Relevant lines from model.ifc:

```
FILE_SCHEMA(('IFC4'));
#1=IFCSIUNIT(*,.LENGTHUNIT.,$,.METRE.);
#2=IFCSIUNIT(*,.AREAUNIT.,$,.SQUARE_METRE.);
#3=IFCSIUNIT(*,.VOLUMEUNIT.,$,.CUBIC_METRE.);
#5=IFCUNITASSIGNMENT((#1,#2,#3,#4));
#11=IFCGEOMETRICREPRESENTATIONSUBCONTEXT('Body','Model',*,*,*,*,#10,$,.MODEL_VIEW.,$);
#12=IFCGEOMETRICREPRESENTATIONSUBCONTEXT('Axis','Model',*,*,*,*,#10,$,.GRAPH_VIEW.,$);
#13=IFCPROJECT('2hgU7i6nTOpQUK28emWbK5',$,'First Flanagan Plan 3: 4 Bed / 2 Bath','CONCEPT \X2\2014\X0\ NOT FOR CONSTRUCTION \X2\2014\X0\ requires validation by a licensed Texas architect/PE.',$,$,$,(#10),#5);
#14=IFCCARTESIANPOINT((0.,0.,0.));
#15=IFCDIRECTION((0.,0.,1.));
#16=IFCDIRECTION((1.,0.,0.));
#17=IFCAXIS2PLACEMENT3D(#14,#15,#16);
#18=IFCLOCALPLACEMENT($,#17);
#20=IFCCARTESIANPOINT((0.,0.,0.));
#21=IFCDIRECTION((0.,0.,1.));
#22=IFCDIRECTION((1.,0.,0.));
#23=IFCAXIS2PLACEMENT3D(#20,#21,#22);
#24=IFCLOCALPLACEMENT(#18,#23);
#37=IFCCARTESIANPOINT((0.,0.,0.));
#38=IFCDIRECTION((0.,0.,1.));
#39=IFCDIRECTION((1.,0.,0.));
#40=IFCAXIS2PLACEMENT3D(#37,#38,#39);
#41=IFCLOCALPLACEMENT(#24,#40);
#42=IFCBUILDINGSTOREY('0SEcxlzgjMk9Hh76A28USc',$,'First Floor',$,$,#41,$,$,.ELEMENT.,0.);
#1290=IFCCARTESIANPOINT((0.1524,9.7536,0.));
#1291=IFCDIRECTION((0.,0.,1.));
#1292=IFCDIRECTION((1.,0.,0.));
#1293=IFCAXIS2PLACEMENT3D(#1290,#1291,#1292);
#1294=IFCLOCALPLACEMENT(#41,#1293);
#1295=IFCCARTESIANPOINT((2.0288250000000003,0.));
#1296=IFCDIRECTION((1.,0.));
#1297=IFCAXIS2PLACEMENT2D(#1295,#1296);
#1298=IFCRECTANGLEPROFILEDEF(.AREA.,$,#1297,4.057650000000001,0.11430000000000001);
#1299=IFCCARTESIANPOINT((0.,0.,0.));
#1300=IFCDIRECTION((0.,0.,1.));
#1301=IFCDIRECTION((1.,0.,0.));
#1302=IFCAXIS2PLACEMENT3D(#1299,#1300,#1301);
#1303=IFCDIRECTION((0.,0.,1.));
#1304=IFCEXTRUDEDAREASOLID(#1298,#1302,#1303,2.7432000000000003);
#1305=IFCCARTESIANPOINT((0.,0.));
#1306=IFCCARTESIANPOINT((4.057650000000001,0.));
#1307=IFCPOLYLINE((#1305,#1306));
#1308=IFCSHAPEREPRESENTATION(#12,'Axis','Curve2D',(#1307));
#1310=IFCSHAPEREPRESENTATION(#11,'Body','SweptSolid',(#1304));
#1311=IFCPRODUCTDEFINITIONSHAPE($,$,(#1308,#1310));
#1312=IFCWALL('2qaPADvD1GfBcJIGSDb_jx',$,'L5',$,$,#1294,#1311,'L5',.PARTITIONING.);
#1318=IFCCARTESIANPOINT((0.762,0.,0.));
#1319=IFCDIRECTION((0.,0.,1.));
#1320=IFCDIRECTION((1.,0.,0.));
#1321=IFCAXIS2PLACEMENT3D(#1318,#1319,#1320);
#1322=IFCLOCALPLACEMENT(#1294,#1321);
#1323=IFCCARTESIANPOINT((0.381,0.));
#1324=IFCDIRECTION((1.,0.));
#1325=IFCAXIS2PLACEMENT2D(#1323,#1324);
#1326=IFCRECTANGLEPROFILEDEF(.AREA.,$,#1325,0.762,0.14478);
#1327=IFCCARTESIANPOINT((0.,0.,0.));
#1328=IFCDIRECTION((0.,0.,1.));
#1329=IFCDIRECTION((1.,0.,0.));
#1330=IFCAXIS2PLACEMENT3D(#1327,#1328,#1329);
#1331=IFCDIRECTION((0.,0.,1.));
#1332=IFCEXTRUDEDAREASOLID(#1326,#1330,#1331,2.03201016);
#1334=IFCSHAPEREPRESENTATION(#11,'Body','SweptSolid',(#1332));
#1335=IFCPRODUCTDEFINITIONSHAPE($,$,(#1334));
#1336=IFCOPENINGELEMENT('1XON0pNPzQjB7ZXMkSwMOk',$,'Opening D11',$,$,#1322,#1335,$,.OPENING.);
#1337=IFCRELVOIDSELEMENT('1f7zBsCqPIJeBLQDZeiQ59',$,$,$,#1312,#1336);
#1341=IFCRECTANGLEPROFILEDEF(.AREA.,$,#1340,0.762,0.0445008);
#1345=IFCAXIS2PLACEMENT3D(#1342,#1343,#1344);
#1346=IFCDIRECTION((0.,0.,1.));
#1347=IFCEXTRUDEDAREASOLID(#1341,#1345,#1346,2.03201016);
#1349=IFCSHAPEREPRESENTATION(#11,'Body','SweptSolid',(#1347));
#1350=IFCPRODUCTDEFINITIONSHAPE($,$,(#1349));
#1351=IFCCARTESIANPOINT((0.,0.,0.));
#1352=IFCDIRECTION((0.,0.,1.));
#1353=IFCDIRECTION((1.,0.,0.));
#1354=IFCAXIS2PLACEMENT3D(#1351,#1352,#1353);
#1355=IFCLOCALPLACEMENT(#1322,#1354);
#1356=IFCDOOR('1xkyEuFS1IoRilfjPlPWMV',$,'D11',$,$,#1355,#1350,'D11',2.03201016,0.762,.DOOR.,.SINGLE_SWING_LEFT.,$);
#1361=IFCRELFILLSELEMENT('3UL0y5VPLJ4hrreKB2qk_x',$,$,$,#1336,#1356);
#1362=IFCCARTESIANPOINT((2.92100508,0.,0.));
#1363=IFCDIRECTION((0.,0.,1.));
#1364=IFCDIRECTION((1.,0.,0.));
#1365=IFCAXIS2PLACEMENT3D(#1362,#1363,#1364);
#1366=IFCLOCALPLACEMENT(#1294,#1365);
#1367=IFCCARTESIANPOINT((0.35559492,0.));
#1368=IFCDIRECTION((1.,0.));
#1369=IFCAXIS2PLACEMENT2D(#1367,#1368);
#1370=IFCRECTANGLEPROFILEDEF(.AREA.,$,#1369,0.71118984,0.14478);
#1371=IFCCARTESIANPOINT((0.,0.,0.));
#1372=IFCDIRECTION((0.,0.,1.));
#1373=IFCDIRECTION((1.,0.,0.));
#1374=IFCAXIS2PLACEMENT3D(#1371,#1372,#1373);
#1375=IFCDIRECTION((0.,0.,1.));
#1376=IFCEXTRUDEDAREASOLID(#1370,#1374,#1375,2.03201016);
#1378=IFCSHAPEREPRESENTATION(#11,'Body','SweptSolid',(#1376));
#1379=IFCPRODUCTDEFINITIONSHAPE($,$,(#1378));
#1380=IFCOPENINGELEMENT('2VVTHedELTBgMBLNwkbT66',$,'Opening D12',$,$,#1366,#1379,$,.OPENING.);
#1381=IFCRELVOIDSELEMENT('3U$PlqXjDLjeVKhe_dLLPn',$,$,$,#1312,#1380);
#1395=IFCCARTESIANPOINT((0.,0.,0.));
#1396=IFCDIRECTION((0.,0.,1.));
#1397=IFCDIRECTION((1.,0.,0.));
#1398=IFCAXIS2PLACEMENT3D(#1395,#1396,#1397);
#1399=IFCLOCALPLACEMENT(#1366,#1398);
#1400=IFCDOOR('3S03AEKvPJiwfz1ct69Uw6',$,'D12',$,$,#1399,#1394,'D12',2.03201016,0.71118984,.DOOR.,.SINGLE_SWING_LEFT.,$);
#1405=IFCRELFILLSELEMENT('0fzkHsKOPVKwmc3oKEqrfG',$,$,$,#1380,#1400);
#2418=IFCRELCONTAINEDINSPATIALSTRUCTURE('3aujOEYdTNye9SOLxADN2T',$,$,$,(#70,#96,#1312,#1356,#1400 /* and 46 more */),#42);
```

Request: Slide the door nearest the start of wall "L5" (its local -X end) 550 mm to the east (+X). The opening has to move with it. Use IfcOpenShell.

```python
import ifcopenshell
import ifcopenshell.api.geometry
import ifcopenshell.util.placement
import ifcopenshell.util.unit

model = ifcopenshell.open("model.ifc")
unit_scale = ifcopenshell.util.unit.calculate_unit_scale(model)

door = model.by_id(1356)
opening = door.FillsVoids[0].RelatingOpeningElement
wall = opening.VoidsElements[0].RelatingBuildingElement

wall_matrix = ifcopenshell.util.placement.get_local_placement(wall.ObjectPlacement)
shift = wall_matrix[:3, 0] * 0.55 / unit_scale
before = ifcopenshell.util.placement.get_local_placement(door.ObjectPlacement)[:3, 3].copy()

# The door is placed relative to its opening, so it follows when the opening moves.
matrix = ifcopenshell.util.placement.get_local_placement(opening.ObjectPlacement)
matrix[:3, 3] += shift
ifcopenshell.api.geometry.edit_object_placement(
    model, product=opening, matrix=matrix, is_si=False, should_transform_children=True
)

after = ifcopenshell.util.placement.get_local_placement(door.ObjectPlacement)[:3, 3]
print("door moved by", (after - before).round(3) + 0.0)

model.write("model_rev.ifc")
```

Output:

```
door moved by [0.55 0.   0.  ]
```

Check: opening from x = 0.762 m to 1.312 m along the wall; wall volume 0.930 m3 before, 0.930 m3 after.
